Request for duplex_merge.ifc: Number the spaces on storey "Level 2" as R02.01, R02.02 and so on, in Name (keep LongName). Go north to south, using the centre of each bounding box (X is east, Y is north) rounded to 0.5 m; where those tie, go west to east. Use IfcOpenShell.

First a look at what the model holds.

```python
import ifcopenshell
import ifcopenshell.util.element
import ifcopenshell.util.placement

model = ifcopenshell.open("duplex_merge.ifc")
print(model.schema)
storey = next(s for s in model.by_type("IfcBuildingStorey") if s.Name == "Level 2")
spaces = [e for e in ifcopenshell.util.element.get_decomposition(storey) if e.is_a("IfcSpace")]
for e in sorted(spaces, key=lambda e: e.id()):
    origin = ifcopenshell.util.placement.get_local_placement(e.ObjectPlacement)[:3, 3]
    print(e.id(), e.Name, e.LongName, origin.round(2) + 0.0, sep=" | ")
```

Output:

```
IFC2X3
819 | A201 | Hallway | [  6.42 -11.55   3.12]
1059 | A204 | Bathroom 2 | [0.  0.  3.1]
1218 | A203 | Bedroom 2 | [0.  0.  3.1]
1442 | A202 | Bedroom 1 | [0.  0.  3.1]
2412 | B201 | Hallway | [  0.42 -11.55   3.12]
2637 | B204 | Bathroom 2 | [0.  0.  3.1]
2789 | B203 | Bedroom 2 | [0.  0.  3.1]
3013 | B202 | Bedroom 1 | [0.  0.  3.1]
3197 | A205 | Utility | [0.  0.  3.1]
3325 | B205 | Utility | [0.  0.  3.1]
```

```python
import ifcopenshell
import ifcopenshell.geom
import ifcopenshell.util.element
import ifcopenshell.util.shape

model = ifcopenshell.open("duplex_merge.ifc")
settings = ifcopenshell.geom.settings()
settings.set("use-world-coords", True)


def centre(element):
    shape = ifcopenshell.geom.create_shape(settings, element)
    return ifcopenshell.util.shape.get_bbox_centroid(shape.geometry)


storey = next(s for s in model.by_type("IfcBuildingStorey") if s.Name == "Level 2")
spaces = [e for e in ifcopenshell.util.element.get_decomposition(storey) if e.is_a("IfcSpace")]

# Insertion points can sit at a corner or the storey origin, so sort by the geometry (in metres).
centres = {e: centre(e) for e in spaces}
spaces.sort(key=lambda e: (-round(centres[e][1] / 0.5), centres[e][0]))

for i, e in enumerate(spaces, start=1):
    number = f"R02.{i:02d}"
    e.Name = number
    print(e.id(), number)

model.write("duplex_merge_v2.ifc")
```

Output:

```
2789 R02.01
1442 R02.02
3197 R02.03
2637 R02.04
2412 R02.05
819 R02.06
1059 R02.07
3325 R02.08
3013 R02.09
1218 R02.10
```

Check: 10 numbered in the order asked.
